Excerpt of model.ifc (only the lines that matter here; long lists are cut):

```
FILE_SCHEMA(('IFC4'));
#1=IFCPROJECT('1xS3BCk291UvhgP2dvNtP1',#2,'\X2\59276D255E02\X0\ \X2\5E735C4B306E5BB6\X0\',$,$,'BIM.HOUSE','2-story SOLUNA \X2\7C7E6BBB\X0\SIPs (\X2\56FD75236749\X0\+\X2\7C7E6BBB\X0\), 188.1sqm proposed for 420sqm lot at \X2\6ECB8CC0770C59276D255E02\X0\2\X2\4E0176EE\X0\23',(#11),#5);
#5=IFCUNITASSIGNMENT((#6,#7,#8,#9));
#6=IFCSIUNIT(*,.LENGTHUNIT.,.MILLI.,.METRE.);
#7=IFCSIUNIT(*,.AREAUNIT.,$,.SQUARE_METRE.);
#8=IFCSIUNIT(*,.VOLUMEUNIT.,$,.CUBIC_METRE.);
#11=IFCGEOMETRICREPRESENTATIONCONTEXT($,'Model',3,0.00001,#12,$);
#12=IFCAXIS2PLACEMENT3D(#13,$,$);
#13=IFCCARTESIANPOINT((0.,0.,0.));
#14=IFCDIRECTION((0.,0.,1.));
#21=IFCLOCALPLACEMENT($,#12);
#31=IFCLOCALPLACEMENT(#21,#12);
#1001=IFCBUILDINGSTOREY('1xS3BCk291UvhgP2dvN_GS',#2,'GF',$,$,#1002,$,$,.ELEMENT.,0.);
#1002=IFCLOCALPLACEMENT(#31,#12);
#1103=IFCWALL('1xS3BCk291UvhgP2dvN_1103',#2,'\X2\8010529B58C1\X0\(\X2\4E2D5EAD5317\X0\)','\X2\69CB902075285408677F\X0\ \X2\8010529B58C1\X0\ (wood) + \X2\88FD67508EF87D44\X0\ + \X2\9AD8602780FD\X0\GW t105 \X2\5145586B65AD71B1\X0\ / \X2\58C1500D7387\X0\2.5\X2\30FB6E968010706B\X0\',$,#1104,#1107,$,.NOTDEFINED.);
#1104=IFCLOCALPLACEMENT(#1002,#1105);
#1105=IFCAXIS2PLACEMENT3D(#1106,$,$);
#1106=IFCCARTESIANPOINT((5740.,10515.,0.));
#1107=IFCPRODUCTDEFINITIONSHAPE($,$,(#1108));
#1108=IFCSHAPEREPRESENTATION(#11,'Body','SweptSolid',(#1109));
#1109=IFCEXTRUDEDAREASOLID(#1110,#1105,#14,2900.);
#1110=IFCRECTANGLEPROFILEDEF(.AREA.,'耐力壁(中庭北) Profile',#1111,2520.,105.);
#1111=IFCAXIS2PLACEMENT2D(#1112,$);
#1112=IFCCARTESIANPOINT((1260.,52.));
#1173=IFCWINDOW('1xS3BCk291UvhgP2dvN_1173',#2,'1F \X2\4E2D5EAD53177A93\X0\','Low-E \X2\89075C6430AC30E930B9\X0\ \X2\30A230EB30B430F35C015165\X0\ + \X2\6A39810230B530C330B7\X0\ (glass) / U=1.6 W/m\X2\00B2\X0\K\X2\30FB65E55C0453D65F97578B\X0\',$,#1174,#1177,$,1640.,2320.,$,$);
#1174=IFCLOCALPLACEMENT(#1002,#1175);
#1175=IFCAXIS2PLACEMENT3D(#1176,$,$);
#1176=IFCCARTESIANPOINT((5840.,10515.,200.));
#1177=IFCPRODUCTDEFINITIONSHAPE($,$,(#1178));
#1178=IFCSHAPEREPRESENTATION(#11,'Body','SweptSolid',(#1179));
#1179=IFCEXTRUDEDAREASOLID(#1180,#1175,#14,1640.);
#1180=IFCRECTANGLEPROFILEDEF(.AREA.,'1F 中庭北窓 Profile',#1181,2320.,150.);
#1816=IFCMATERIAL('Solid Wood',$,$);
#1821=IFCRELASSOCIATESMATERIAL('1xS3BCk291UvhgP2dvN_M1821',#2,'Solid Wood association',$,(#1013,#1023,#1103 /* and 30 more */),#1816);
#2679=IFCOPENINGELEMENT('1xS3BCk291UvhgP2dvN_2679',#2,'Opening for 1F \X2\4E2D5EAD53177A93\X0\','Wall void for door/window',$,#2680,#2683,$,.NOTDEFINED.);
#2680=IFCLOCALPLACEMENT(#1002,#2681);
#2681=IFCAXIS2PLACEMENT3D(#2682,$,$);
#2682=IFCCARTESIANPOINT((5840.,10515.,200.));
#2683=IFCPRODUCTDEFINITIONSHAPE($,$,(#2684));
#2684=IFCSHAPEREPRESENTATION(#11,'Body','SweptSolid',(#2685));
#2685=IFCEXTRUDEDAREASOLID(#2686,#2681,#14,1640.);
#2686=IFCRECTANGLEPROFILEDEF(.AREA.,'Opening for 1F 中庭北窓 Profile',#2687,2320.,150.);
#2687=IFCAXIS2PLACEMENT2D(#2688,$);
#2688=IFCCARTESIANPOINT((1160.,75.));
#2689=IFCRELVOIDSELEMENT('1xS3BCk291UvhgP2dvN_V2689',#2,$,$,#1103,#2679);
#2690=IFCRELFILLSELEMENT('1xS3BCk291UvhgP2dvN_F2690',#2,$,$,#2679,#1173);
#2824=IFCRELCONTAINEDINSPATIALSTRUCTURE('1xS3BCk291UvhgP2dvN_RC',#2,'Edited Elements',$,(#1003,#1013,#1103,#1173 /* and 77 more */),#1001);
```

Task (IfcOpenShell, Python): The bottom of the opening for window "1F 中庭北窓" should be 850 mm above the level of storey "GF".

```python
import numpy as np
import ifcopenshell
import ifcopenshell.api.geometry
import ifcopenshell.geom
import ifcopenshell.util.element
import ifcopenshell.util.placement
import ifcopenshell.util.shape
import ifcopenshell.util.unit

model = ifcopenshell.open("model.ifc")
unit_scale = ifcopenshell.util.unit.calculate_unit_scale(model)

window = model.by_guid("1xS3BCk291UvhgP2dvN_1173")
opening = window.FillsVoids[0].RelatingOpeningElement
storey = ifcopenshell.util.element.get_container(window, ifc_class="IfcBuildingStorey")
level = ifcopenshell.util.placement.get_local_placement(storey.ObjectPlacement)[2, 3]

# The opening's origin need not be at the sill, so measure its lowest point.
shape = ifcopenshell.geom.create_shape(ifcopenshell.geom.settings(), opening)
bottom = ifcopenshell.util.shape.get_shape_bottom_elevation(shape, shape.geometry) / unit_scale
dz = level + 850.0 - bottom

shift = np.array([0.0, 0.0, dz])
# The window is not placed relative to its opening, so move both.
for product in (opening, window):
    matrix = ifcopenshell.util.placement.get_local_placement(product.ObjectPlacement)
    matrix[:3, 3] += shift
    ifcopenshell.api.geometry.edit_object_placement(model, product=product, matrix=matrix, is_si=False)

print(f"moved by {dz * unit_scale:+.3f} m")

model.write("model_updated.ifc")
```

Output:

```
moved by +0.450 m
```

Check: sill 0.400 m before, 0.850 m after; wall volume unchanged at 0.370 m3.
